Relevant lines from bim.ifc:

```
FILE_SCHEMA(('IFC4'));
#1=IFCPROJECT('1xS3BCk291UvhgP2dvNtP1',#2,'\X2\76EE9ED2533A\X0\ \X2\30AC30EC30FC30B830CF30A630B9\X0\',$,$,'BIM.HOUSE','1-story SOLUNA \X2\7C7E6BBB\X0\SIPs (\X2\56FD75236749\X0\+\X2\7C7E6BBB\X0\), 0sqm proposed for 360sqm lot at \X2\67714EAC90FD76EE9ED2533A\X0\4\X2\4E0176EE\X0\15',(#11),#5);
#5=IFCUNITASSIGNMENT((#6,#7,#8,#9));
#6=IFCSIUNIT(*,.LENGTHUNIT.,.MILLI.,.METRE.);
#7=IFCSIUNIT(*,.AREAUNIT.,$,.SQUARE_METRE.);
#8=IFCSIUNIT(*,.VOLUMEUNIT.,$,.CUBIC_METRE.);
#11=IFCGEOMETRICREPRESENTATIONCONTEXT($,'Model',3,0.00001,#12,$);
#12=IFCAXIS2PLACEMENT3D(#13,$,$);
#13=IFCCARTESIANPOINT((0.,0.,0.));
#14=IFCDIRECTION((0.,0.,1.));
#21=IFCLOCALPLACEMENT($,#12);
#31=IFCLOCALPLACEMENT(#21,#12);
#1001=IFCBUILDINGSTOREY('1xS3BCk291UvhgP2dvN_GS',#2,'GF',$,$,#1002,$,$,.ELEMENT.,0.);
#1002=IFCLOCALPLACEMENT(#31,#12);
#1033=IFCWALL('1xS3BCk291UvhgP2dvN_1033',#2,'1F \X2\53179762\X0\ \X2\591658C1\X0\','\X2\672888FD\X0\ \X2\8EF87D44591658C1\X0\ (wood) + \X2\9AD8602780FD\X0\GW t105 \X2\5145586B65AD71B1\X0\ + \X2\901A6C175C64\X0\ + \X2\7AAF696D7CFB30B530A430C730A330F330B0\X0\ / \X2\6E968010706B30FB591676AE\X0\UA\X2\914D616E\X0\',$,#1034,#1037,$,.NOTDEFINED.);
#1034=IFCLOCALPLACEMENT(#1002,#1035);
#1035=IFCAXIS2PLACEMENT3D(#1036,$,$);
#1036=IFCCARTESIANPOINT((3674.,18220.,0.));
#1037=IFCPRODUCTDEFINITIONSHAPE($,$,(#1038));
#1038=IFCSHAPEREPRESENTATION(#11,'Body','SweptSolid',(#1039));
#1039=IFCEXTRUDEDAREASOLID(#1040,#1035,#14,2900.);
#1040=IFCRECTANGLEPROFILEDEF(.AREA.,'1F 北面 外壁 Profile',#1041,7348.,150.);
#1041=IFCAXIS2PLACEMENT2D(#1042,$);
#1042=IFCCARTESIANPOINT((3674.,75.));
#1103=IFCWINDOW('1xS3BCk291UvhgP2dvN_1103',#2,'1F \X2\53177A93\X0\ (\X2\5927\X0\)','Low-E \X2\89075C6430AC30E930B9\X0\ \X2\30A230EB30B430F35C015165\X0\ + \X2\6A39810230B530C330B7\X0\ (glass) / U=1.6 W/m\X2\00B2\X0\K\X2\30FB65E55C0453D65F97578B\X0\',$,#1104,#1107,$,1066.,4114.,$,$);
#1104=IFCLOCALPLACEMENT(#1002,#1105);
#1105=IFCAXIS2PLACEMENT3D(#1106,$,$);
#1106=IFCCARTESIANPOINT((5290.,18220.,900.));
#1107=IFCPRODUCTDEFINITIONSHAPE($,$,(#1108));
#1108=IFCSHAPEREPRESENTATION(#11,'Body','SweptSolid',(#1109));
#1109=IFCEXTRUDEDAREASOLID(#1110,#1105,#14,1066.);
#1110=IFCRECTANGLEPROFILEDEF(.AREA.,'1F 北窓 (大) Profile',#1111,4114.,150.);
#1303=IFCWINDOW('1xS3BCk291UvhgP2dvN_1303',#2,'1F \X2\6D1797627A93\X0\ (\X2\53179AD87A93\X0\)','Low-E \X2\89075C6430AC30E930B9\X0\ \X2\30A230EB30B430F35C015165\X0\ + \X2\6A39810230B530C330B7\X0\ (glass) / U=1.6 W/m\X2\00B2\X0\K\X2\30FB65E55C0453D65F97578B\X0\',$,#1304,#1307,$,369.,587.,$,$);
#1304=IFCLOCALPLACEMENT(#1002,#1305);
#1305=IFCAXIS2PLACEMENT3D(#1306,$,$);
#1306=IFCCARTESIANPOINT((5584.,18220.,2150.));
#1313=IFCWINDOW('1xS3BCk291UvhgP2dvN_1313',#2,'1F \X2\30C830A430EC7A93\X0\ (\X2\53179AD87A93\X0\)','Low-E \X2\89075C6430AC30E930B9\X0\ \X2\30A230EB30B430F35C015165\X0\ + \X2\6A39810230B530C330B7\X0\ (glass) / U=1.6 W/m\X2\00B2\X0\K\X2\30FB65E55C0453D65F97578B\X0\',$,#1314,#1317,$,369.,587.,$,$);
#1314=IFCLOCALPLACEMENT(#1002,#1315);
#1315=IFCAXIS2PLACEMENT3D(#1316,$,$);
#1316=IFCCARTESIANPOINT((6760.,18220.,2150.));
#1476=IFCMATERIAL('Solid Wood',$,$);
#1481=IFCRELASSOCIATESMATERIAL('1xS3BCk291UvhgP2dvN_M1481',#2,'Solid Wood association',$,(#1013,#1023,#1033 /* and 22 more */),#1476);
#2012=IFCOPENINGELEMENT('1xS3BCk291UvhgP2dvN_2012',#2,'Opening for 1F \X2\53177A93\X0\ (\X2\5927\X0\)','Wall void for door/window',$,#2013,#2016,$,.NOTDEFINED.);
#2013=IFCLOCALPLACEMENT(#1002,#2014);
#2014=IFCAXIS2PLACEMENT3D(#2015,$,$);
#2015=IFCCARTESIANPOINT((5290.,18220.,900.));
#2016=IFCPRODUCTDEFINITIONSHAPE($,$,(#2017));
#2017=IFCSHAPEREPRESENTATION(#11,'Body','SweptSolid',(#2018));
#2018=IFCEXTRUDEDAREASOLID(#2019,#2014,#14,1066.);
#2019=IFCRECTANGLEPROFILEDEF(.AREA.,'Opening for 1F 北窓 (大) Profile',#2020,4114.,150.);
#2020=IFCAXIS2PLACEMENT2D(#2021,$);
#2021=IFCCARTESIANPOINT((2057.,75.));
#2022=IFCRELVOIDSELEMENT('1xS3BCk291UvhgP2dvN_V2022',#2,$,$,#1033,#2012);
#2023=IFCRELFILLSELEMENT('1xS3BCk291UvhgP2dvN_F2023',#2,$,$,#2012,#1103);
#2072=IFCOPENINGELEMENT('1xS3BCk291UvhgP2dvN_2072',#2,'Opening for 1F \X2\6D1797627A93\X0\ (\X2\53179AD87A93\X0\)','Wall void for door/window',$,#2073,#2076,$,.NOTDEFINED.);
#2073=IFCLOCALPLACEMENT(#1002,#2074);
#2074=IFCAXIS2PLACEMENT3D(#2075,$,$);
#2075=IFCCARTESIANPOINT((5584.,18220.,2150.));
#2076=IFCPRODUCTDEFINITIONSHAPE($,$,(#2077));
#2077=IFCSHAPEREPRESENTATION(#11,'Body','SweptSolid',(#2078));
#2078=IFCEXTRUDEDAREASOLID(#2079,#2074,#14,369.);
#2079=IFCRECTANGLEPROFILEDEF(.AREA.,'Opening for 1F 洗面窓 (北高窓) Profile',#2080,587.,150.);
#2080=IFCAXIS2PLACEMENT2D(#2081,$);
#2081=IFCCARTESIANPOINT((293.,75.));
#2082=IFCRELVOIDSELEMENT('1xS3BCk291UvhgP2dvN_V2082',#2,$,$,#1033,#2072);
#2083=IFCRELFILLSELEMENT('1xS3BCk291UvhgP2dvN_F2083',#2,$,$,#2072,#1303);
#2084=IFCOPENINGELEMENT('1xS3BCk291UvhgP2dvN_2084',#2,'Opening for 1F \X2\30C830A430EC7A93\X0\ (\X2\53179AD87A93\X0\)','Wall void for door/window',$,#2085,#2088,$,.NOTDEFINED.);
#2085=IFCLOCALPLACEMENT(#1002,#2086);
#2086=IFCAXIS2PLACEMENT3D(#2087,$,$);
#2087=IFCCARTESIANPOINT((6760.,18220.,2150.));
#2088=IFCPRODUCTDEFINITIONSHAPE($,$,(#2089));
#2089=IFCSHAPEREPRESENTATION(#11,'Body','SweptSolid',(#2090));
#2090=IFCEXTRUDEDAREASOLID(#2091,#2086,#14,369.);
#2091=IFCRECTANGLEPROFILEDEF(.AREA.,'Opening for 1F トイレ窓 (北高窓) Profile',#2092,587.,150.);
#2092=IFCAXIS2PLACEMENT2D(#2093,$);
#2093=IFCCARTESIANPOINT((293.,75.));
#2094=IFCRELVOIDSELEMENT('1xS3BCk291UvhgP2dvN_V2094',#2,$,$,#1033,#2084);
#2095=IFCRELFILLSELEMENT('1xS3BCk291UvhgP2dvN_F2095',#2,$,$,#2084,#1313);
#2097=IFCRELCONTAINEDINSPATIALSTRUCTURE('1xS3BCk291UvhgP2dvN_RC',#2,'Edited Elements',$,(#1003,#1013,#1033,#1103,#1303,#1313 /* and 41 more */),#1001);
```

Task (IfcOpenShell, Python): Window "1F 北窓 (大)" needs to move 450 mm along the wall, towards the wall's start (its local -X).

```python
import ifcopenshell
import ifcopenshell.api.geometry
import ifcopenshell.util.placement

model = ifcopenshell.open("bim.ifc")

window = model.by_guid("1xS3BCk291UvhgP2dvN_1103")
opening = window.FillsVoids[0].RelatingOpeningElement
wall = opening.VoidsElements[0].RelatingBuildingElement

wall_matrix = ifcopenshell.util.placement.get_local_placement(wall.ObjectPlacement)
shift = wall_matrix[:3, 0] * -450.0
before = ifcopenshell.util.placement.get_local_placement(window.ObjectPlacement)[:3, 3].copy()

# The window is not placed relative to its opening, so move both.
for product in (opening, window):
    matrix = ifcopenshell.util.placement.get_local_placement(product.ObjectPlacement)
    matrix[:3, 3] += shift
    ifcopenshell.api.geometry.edit_object_placement(model, product=product, matrix=matrix, is_si=False)

after = ifcopenshell.util.placement.get_local_placement(window.ObjectPlacement)[:3, 3]
print("window moved by", (after - before).round(3) + 0.0)

model.write("bim_v2.ifc")
```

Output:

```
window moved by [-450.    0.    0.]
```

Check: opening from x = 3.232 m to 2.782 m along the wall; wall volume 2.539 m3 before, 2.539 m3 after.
